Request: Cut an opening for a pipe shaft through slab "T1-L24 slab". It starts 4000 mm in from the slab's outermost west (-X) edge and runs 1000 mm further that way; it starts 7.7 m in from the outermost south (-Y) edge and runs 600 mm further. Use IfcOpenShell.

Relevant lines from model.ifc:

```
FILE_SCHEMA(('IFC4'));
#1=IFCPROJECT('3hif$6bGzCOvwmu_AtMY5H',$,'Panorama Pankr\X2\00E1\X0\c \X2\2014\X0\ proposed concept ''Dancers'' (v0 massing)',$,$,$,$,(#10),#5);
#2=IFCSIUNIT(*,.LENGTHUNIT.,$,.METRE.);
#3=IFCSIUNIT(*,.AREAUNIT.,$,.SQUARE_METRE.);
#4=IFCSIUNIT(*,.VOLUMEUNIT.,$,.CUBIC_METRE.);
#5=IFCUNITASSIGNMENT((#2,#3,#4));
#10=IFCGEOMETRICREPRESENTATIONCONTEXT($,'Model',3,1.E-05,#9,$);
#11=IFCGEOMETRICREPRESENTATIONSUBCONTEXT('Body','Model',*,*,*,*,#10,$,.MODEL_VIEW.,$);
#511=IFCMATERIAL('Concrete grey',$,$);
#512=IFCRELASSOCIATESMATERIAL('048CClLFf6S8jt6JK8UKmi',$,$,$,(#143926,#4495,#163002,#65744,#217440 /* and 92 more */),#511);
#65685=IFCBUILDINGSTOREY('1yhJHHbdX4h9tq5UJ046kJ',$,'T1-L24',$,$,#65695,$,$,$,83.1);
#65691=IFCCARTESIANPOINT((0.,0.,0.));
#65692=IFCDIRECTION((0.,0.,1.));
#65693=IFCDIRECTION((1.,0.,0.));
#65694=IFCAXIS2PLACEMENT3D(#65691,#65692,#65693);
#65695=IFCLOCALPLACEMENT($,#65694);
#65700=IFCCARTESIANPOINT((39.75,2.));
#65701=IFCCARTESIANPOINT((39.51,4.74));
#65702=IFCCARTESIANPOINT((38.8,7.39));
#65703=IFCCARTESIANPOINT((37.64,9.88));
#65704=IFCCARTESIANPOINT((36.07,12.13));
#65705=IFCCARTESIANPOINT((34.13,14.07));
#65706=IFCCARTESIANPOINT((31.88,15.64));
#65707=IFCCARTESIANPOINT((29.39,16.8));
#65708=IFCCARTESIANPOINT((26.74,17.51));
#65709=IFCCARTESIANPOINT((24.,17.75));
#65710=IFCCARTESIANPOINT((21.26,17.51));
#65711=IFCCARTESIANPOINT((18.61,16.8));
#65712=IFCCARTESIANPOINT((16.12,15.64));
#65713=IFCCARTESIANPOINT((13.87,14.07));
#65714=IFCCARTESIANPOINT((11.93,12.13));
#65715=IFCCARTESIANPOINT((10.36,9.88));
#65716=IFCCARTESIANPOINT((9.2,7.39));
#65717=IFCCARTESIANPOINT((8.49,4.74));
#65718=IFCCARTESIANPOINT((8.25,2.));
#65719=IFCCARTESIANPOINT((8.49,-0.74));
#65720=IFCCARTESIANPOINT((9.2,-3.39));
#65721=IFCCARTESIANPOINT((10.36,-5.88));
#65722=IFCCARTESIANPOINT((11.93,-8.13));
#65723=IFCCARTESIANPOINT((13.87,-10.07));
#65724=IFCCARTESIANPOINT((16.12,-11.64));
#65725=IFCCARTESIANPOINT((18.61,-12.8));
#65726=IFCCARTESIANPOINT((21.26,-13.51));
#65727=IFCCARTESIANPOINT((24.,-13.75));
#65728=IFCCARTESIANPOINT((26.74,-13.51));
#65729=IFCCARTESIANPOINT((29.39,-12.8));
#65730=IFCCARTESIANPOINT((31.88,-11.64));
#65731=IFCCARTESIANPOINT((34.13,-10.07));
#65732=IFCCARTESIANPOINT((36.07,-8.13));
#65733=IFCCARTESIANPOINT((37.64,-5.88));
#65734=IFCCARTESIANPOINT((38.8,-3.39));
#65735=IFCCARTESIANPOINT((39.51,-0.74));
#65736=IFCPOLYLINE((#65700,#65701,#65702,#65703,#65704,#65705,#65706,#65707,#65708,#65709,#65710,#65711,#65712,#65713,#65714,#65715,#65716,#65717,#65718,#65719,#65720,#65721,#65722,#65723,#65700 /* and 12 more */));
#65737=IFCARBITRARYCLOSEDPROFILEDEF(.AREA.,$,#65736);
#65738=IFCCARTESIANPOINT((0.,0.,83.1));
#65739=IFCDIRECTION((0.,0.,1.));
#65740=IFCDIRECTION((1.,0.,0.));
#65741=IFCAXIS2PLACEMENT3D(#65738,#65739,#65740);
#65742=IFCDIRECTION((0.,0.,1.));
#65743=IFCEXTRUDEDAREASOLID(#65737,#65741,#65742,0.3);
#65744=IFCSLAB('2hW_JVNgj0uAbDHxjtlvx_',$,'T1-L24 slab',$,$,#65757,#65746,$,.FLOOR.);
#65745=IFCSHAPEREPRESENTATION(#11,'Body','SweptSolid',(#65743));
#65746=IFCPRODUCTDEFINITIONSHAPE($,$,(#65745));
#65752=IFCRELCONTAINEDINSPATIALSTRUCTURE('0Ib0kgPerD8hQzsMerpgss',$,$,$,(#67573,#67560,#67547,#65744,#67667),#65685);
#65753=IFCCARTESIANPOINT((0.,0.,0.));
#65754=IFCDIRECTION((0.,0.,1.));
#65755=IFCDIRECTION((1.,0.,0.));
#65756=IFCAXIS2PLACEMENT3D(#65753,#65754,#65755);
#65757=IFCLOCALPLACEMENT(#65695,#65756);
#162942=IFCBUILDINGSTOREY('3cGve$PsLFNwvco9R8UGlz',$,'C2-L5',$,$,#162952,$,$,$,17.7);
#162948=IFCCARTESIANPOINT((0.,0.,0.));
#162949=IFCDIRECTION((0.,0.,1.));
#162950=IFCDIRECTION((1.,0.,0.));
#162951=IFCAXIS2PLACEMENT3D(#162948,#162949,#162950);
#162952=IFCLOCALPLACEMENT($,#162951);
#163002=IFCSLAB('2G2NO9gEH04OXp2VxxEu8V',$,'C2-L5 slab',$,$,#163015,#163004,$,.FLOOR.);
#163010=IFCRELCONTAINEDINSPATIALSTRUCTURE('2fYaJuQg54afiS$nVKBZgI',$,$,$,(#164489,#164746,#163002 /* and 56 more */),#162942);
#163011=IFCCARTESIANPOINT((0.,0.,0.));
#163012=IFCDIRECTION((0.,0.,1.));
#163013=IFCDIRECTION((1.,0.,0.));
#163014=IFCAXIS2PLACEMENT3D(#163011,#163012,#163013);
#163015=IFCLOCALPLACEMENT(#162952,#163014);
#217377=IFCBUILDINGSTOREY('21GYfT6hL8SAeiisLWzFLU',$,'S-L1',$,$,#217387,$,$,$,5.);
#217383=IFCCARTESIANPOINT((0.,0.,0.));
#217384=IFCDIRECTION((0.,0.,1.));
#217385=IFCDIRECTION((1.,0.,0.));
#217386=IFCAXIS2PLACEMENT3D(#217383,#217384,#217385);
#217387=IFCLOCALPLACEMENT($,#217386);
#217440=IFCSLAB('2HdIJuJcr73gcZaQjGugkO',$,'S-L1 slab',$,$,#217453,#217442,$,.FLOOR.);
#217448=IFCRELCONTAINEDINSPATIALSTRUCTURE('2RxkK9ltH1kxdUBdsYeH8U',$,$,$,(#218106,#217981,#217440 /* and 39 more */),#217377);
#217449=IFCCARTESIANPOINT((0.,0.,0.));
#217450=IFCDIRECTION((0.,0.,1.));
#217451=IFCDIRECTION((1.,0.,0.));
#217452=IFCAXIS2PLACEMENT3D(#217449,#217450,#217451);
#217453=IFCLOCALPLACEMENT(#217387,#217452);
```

```python
import numpy as np
import ifcopenshell
import ifcopenshell.api.feature
import ifcopenshell.api.geometry
import ifcopenshell.api.root
import ifcopenshell.geom
import ifcopenshell.util.placement
import ifcopenshell.util.representation
import ifcopenshell.util.shape
import ifcopenshell.util.unit

model = ifcopenshell.open("model.ifc")
unit_scale = ifcopenshell.util.unit.calculate_unit_scale(model)
settings = ifcopenshell.geom.settings()


def volume(element):
    """Net volume in cubic metres, openings subtracted."""
    shape = ifcopenshell.geom.create_shape(settings, element)
    return ifcopenshell.util.shape.get_volume(shape.geometry)


slab = model.by_guid("2hW_JVNgj0uAbDHxjtlvx_")
before = volume(slab)

# Extent in the slab's own axes, in metres. The edges named are its -X and -Y sides.
slab_shape = ifcopenshell.geom.create_shape(settings, slab)
vertices = ifcopenshell.util.shape.get_vertices(slab_shape.geometry)
x_min, y_min, bottom = vertices.min(axis=0)
top = vertices[:, 2].max()

opening = ifcopenshell.api.root.create_entity(model, ifc_class="IfcOpeningElement", name="Pipe shaft opening", predefined_type="OPENING")
context = ifcopenshell.util.representation.get_context(model, "Model", "Body", "MODEL_VIEW")
width, depth = 1, 0.6
outline = [(0.0, 0.0), (width, 0.0), (width, depth), (0.0, depth), (0.0, 0.0)]
# Overshoot both faces by 50 mm so the cut is clean.
shape = ifcopenshell.api.geometry.add_slab_representation(
    model, context=context, depth=top - bottom + 0.1, polyline=outline
)
ifcopenshell.api.geometry.assign_representation(model, product=opening, representation=shape)

matrix = ifcopenshell.util.placement.get_local_placement(slab.ObjectPlacement)
matrix[:, 3] = matrix @ np.append(np.array([x_min + 4, y_min + 7.7, bottom - 0.05]) / unit_scale, 1.0)
ifcopenshell.api.geometry.edit_object_placement(model, product=opening, matrix=matrix, is_si=False)
ifcopenshell.api.feature.add_feature(model, feature=opening, element=slab)

after = volume(slab)

print(f"slab volume {before:.3f} -> {after:.3f} m3")

model.write("model_updated.ifc")
```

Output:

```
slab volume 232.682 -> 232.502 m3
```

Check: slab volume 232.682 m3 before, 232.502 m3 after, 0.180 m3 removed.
